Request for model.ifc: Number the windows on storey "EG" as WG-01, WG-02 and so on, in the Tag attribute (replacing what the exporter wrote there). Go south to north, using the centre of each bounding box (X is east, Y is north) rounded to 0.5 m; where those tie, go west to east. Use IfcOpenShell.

First a look at what the model holds.

```python
import ifcopenshell
import ifcopenshell.util.element
import ifcopenshell.util.placement

model = ifcopenshell.open("model.ifc")
print(model.schema)
storey = next(s for s in model.by_type("IfcBuildingStorey") if s.Name == "EG")
windows = [e for e in ifcopenshell.util.element.get_decomposition(storey) if e.is_a("IfcWindow")]
for e in sorted(windows, key=lambda e: e.id()):
    origin = ifcopenshell.util.placement.get_local_placement(e.ObjectPlacement)[:3, 3]
    print(e.id(), e.Tag, e.Name, origin.round(2) + 0.0, sep=" | ")
```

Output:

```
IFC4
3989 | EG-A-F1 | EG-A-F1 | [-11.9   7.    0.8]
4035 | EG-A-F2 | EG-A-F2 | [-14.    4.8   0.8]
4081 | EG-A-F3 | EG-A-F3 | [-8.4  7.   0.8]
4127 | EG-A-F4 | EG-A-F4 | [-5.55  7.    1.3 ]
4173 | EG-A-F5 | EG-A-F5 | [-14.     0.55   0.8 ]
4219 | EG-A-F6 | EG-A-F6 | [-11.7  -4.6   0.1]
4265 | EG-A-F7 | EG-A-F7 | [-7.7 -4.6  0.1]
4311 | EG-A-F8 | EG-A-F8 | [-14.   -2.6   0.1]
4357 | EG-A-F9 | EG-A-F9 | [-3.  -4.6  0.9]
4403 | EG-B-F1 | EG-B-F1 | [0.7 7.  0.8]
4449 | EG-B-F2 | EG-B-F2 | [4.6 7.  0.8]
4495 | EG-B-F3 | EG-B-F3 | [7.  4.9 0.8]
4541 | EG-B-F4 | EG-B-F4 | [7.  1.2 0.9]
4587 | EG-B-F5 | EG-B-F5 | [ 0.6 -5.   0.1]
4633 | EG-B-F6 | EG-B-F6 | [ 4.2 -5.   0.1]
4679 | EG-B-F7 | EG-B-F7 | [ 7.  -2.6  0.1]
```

```python
import ifcopenshell
import ifcopenshell.geom
import ifcopenshell.util.element
import ifcopenshell.util.shape

model = ifcopenshell.open("model.ifc")
settings = ifcopenshell.geom.settings()
settings.set("use-world-coords", True)


def centre(element):
    shape = ifcopenshell.geom.create_shape(settings, element)
    return ifcopenshell.util.shape.get_bbox_centroid(shape.geometry)


storey = next(s for s in model.by_type("IfcBuildingStorey") if s.Name == "EG")
windows = [e for e in ifcopenshell.util.element.get_decomposition(storey) if e.is_a("IfcWindow")]

# Insertion points can sit at a corner or the storey origin, so sort by the geometry (in metres).
centres = {e: centre(e) for e in windows}
windows.sort(key=lambda e: (round(centres[e][1] / 0.5), centres[e][0]))

for i, e in enumerate(windows, start=1):
    number = f"WG-{i:02d}"
    e.Tag = number
    print(e.id(), number)

model.write("model-out.ifc")
```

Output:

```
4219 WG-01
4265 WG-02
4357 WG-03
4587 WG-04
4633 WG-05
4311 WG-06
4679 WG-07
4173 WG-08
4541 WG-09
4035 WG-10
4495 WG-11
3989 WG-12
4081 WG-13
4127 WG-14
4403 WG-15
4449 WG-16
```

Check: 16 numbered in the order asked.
